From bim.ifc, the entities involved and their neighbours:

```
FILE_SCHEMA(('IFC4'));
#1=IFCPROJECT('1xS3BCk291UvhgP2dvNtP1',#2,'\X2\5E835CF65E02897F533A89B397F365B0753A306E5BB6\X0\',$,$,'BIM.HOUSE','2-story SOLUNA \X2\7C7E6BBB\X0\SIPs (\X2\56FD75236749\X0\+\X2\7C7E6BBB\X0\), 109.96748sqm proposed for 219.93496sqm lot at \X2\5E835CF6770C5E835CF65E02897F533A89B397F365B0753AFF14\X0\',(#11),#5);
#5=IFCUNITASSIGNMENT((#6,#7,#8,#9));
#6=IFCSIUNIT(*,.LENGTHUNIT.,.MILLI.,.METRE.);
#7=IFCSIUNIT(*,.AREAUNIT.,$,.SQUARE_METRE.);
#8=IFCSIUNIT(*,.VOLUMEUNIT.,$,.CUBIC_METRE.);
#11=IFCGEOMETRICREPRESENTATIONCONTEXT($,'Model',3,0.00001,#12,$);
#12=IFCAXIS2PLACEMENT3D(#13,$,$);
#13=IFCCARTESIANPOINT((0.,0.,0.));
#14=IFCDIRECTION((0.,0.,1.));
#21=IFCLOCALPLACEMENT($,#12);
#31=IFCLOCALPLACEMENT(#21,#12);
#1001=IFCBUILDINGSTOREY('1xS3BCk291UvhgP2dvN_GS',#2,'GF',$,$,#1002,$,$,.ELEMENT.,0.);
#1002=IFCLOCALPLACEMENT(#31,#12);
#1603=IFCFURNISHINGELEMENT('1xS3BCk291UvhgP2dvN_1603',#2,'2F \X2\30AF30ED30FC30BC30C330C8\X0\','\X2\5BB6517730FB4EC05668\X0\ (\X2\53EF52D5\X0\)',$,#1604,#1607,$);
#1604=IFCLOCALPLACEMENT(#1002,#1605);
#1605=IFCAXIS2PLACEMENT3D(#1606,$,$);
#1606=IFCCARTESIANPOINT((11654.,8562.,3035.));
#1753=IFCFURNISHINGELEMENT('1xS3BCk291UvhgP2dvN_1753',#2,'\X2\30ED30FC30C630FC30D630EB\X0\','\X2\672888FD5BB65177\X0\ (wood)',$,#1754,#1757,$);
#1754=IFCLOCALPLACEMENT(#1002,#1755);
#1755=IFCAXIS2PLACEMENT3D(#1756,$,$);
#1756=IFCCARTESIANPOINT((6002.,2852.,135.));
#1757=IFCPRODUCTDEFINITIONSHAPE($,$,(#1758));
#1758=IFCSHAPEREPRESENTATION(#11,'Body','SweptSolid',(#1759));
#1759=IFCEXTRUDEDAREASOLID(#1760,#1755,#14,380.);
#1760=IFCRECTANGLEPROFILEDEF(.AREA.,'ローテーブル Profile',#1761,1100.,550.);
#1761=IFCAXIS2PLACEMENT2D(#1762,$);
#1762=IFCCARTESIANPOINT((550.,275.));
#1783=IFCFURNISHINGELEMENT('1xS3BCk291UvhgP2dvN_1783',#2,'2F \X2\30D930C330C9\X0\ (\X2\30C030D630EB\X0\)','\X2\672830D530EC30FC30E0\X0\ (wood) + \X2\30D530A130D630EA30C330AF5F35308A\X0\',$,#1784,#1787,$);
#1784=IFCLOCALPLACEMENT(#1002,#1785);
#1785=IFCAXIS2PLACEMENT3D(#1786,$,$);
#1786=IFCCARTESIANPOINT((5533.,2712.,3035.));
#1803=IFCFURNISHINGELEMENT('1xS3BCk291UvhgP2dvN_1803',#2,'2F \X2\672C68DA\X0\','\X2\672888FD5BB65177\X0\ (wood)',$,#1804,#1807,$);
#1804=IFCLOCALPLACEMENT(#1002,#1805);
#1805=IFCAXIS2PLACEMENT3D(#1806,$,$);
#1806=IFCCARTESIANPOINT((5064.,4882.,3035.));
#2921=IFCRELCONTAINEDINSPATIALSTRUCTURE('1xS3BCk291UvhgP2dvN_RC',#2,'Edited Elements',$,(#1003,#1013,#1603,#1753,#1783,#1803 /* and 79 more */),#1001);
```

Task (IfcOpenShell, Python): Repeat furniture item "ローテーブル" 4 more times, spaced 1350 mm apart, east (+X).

```python
import numpy as np
import ifcopenshell
import ifcopenshell.api.geometry
import ifcopenshell.api.root
import ifcopenshell.util.element
import ifcopenshell.util.placement

model = ifcopenshell.open("bim.ifc")


def reuse_history(source, copy):
    """copy_class also copies each property set's owner history, people and application; keep the originals."""
    for rel in copy.IsDefinedBy:
        if rel.is_a("IfcRelDefinesByProperties") and (history := rel.RelatingPropertyDefinition.OwnerHistory):
            rel.RelatingPropertyDefinition.OwnerHistory = source.OwnerHistory
            ifcopenshell.util.element.remove_deep2(model, history)


source = model.by_guid("1xS3BCk291UvhgP2dvN_1753")
base = ifcopenshell.util.placement.get_local_placement(source.ObjectPlacement)
step = np.array([1.0, 0.0, 0.0]) * 1350.0

for i in range(1, 5):
    copy = ifcopenshell.api.root.copy_class(model, product=source)
    copy.Representation = ifcopenshell.util.element.copy_deep(
        model, source.Representation, exclude=["IfcGeometricRepresentationContext", "IfcRepresentationMap"]
    )
    reuse_history(source, copy)
    matrix = base.copy()
    matrix[:3, 3] += i * step
    print("added at", matrix[:3, 3].round(3) + 0.0)
    ifcopenshell.api.geometry.edit_object_placement(model, product=copy, matrix=matrix, is_si=False)

model.write("bim_v2.ifc")
```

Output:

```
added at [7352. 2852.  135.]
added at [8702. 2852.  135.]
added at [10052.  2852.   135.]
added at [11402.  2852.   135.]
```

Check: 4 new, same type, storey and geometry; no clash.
